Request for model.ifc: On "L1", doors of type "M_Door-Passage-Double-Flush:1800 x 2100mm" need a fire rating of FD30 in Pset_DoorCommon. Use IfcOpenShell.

First a look at what the model holds.

```python
import ifcopenshell
import ifcopenshell.util.element

model = ifcopenshell.open("model.ifc")
print(model.schema)
storey = next(s for s in model.by_type("IfcBuildingStorey") if s.Name == "L1")
doors = [e for e in ifcopenshell.util.element.get_decomposition(storey) if e.is_a("IfcDoor")]
seen = {}
for e in doors:
    element_type = ifcopenshell.util.element.get_type(e)
    key = (element_type.Name if element_type != e and element_type else None, ifcopenshell.util.element.get_pset(e, "Pset_DoorCommon", "FireRating"))
    seen[key] = seen.get(key, 0) + 1
for (name, value), count in sorted(seen.items(), key=str):
    print(count, "x", name, "|", value)
```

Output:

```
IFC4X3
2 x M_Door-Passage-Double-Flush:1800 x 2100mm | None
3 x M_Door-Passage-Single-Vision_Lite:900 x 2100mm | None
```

```python
import ifcopenshell
import ifcopenshell.api.pset
import ifcopenshell.util.element

model = ifcopenshell.open("model.ifc")

storey = next(s for s in model.by_type("IfcBuildingStorey") if s.Name == "L1")
doors = [e for e in ifcopenshell.util.element.get_decomposition(storey) if e.is_a("IfcDoor")]

count = 0
for e in doors:
    element_type = ifcopenshell.util.element.get_type(e)
    if element_type in (None, e) or element_type.Name != "M_Door-Passage-Double-Flush:1800 x 2100mm":
        continue
    # add_pset returns the element's existing set when there is one.
    pset = ifcopenshell.api.pset.add_pset(model, product=e, name="Pset_DoorCommon")
    ifcopenshell.api.pset.edit_pset(model, pset=pset, properties={"FireRating": "FD30"})
    count += 1

print(count, "doors updated")

model.write("model_edited.ifc")
```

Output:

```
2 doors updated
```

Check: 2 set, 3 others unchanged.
